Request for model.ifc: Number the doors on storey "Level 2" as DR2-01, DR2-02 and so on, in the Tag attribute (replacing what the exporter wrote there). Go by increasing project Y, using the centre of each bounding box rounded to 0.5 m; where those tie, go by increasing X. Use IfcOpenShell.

First a look at what the model holds.

```python
import ifcopenshell
import ifcopenshell.util.element
import ifcopenshell.util.placement

model = ifcopenshell.open("model.ifc")
print(model.schema)
storey = next(s for s in model.by_type("IfcBuildingStorey") if s.Name == "Level 2")
doors = [e for e in ifcopenshell.util.element.get_decomposition(storey) if e.is_a("IfcDoor")]
for e in sorted(doors, key=lambda e: e.id()):
    origin = ifcopenshell.util.placement.get_local_placement(e.ObjectPlacement)[:3, 3]
    print(e.id(), e.Tag, e.Name, origin.round(2) + 0.0, sep=" | ")
```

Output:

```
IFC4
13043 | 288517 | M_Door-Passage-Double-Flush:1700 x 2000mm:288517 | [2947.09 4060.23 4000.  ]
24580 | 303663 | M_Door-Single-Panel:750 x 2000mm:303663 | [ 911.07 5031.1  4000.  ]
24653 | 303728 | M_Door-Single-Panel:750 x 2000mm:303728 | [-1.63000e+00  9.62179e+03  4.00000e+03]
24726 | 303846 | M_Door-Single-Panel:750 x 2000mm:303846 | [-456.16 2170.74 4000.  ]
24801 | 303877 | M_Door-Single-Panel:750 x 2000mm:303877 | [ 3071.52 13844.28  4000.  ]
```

```python
import ifcopenshell
import ifcopenshell.geom
import ifcopenshell.util.element
import ifcopenshell.util.shape

model = ifcopenshell.open("model.ifc")
settings = ifcopenshell.geom.settings()
settings.set("use-world-coords", True)


def centre(element):
    shape = ifcopenshell.geom.create_shape(settings, element)
    return ifcopenshell.util.shape.get_bbox_centroid(shape.geometry)


storey = next(s for s in model.by_type("IfcBuildingStorey") if s.Name == "Level 2")
doors = [e for e in ifcopenshell.util.element.get_decomposition(storey) if e.is_a("IfcDoor")]

# Insertion points can sit at a corner or the storey origin, so sort by the geometry (in metres).
centres = {e: centre(e) for e in doors}
doors.sort(key=lambda e: (round(centres[e][1] / 0.5), centres[e][0]))

for i, e in enumerate(doors, start=1):
    number = f"DR2-{i:02d}"
    e.Tag = number
    print(e.id(), number)

model.write("model_edited.ifc")
```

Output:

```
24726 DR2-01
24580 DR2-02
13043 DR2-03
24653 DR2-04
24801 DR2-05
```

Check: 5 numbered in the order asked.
